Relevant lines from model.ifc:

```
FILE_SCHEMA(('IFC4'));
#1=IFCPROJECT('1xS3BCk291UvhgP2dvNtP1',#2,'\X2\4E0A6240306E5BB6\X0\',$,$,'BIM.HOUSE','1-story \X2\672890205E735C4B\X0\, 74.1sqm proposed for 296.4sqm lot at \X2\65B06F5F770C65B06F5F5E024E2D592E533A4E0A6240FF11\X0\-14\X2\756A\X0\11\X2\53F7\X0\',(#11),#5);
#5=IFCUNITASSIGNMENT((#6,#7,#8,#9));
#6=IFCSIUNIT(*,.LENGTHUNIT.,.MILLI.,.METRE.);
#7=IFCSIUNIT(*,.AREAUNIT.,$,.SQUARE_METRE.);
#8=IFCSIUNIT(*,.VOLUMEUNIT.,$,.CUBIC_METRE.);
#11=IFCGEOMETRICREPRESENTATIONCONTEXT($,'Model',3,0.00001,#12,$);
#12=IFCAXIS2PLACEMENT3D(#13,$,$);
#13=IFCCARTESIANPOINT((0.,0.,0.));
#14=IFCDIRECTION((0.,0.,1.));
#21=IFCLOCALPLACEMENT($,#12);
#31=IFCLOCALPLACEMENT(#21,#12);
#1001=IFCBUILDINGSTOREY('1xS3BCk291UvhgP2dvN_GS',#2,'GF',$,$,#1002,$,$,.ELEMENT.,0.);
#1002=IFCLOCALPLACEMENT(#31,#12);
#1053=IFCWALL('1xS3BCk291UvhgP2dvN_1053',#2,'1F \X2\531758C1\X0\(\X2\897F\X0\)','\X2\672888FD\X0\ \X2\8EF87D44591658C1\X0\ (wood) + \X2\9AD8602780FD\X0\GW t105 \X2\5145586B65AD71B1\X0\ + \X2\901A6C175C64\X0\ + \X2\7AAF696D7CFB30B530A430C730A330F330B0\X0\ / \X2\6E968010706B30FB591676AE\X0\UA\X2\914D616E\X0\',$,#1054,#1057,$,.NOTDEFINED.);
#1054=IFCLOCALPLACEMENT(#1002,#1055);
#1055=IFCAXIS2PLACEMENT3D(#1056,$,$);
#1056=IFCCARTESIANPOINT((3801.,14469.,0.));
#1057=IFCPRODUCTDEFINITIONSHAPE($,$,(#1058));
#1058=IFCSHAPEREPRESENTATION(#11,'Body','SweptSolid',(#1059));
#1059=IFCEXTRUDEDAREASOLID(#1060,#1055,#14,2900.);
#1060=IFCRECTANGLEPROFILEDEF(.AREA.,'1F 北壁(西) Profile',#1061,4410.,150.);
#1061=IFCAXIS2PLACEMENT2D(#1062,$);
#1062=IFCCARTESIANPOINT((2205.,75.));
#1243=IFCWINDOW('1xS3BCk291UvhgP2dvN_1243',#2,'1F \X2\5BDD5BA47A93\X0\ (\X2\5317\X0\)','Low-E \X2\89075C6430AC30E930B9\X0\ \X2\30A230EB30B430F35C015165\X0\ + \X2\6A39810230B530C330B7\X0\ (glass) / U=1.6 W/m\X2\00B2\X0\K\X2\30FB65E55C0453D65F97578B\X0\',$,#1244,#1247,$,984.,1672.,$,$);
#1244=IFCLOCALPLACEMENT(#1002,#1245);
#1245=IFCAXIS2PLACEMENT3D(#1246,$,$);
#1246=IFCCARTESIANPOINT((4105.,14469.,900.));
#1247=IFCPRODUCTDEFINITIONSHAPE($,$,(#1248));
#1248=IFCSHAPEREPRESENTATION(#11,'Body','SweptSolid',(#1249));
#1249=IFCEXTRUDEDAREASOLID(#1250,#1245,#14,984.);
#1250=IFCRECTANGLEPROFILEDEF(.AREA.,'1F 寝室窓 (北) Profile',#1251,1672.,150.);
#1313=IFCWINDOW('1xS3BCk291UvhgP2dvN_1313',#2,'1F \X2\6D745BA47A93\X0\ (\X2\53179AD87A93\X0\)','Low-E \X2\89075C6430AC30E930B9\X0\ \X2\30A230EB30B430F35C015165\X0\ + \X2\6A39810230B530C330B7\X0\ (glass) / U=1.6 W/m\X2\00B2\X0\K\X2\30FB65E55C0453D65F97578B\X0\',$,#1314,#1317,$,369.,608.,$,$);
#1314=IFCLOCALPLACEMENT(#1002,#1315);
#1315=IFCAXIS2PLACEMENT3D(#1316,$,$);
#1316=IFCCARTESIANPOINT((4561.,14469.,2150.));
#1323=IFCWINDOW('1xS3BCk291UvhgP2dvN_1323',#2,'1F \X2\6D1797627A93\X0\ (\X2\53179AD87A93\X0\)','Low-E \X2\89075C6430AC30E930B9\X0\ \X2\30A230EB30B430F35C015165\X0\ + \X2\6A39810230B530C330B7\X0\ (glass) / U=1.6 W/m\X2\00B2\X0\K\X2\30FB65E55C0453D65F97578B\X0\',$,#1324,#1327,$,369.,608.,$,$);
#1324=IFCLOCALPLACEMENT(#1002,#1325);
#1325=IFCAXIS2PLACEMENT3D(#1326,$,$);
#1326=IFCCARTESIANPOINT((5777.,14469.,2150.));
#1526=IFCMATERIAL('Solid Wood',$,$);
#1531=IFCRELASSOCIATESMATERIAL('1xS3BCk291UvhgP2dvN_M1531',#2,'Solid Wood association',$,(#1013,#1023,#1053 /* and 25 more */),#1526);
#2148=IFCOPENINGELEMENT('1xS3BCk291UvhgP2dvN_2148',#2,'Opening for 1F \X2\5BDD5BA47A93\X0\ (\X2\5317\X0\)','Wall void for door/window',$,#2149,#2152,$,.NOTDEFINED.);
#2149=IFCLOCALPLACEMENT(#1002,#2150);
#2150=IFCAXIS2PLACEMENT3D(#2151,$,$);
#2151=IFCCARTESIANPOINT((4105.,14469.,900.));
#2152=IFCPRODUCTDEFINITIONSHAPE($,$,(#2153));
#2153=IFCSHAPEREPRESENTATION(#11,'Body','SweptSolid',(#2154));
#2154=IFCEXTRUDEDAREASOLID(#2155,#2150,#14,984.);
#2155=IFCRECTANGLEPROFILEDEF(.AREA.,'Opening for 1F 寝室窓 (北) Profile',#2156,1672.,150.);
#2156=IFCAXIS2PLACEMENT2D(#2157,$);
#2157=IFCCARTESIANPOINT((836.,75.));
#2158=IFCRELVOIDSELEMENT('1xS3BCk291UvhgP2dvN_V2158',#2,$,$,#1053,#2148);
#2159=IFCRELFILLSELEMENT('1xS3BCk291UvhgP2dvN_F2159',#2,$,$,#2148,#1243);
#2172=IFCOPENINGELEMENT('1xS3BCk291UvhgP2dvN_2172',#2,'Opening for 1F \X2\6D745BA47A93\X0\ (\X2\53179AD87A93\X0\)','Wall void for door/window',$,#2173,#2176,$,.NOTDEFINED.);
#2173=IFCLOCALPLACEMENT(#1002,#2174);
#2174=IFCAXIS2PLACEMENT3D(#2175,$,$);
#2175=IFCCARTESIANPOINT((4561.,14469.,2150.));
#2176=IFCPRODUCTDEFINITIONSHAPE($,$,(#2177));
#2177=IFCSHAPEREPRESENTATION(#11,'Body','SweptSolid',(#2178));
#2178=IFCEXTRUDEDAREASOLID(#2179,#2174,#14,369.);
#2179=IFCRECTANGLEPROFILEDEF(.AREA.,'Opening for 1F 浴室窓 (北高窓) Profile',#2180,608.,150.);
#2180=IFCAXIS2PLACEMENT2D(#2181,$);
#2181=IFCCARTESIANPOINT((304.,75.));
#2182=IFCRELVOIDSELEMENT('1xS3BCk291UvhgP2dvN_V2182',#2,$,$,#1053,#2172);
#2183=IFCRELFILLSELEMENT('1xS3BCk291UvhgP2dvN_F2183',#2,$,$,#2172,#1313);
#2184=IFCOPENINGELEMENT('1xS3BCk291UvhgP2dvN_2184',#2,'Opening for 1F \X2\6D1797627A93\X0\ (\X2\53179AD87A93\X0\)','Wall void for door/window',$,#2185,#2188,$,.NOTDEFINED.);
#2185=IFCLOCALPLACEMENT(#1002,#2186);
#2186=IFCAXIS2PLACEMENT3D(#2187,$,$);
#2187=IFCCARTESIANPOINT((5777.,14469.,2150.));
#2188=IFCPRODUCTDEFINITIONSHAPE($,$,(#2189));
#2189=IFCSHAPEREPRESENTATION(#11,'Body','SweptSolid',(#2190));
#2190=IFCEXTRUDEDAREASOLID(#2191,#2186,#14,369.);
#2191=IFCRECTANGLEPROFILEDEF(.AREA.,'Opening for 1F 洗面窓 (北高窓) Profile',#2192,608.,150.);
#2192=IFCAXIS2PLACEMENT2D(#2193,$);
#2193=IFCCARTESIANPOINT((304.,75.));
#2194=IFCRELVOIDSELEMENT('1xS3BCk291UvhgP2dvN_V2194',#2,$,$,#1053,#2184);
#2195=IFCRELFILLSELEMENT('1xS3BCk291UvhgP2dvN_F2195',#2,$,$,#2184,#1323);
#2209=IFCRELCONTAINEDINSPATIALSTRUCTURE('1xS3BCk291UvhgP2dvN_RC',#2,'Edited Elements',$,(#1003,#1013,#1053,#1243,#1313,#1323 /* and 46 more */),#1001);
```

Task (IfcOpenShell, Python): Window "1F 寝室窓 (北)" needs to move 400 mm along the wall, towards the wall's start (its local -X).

```python
import ifcopenshell
import ifcopenshell.api.geometry
import ifcopenshell.util.placement
import ifcopenshell.util.unit

model = ifcopenshell.open("model.ifc")
unit_scale = ifcopenshell.util.unit.calculate_unit_scale(model)

window = model.by_guid("1xS3BCk291UvhgP2dvN_1243")
opening = window.FillsVoids[0].RelatingOpeningElement
wall = opening.VoidsElements[0].RelatingBuildingElement

wall_matrix = ifcopenshell.util.placement.get_local_placement(wall.ObjectPlacement)
shift = wall_matrix[:3, 0] * -0.4 / unit_scale
before = ifcopenshell.util.placement.get_local_placement(window.ObjectPlacement)[:3, 3].copy()

# The window is not placed relative to its opening, so move both.
for product in (opening, window):
    matrix = ifcopenshell.util.placement.get_local_placement(product.ObjectPlacement)
    matrix[:3, 3] += shift
    ifcopenshell.api.geometry.edit_object_placement(model, product=product, matrix=matrix, is_si=False)

after = ifcopenshell.util.placement.get_local_placement(window.ObjectPlacement)[:3, 3]
print("window moved by", (after - before).round(3) + 0.0)

model.write("model_updated.ifc")
```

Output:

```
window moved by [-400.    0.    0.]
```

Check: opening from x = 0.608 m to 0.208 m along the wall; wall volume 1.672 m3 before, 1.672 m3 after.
